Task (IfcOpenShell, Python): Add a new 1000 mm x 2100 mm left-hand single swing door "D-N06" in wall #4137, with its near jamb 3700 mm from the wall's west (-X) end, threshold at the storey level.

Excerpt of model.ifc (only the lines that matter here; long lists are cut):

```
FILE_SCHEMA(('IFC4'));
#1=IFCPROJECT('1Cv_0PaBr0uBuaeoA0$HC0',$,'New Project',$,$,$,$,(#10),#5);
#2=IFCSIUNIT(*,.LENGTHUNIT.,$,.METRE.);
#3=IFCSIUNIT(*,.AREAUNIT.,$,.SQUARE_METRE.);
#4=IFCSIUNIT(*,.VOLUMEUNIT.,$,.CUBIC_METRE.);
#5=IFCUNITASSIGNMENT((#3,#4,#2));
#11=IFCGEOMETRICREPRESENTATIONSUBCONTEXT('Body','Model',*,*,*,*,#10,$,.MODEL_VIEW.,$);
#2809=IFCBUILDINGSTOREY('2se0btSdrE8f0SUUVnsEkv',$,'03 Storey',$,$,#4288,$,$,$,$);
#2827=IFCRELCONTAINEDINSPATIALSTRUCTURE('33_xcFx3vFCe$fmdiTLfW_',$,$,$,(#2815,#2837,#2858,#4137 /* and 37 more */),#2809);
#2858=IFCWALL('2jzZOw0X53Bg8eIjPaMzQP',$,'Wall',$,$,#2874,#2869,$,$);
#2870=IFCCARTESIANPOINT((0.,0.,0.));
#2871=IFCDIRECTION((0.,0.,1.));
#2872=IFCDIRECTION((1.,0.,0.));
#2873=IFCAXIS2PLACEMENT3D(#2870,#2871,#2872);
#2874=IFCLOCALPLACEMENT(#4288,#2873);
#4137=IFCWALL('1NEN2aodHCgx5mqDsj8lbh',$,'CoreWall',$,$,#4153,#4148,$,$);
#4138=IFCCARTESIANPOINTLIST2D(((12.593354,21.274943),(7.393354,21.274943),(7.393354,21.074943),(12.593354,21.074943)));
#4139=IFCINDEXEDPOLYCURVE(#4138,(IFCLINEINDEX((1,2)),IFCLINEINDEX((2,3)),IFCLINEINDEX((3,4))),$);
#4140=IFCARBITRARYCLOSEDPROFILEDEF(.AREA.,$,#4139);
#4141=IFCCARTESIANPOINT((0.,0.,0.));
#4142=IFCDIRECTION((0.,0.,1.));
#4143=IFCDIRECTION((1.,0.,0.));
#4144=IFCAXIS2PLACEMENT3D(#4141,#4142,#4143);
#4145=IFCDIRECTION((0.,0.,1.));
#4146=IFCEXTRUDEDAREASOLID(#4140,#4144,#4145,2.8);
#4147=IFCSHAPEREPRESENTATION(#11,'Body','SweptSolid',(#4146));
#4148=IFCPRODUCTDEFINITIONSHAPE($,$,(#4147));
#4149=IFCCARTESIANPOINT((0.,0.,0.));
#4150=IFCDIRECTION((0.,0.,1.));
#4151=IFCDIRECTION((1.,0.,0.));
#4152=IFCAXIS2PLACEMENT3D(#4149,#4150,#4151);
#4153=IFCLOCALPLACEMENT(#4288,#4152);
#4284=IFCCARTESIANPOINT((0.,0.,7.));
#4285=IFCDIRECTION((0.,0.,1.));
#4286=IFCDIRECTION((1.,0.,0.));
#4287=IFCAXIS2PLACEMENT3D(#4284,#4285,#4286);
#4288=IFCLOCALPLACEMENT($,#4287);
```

```python
import numpy as np
import ifcopenshell
import ifcopenshell.api.feature
import ifcopenshell.api.geometry
import ifcopenshell.api.root
import ifcopenshell.api.spatial
import ifcopenshell.geom
import ifcopenshell.util.element
import ifcopenshell.util.placement
import ifcopenshell.util.representation
import ifcopenshell.util.shape
import ifcopenshell.util.unit

model = ifcopenshell.open("model.ifc")
unit_scale = ifcopenshell.util.unit.calculate_unit_scale(model)
settings = ifcopenshell.geom.settings()


def volume(element):
    """Net volume in cubic metres, openings subtracted."""
    shape = ifcopenshell.geom.create_shape(settings, element)
    return ifcopenshell.util.shape.get_volume(shape.geometry)


wall = model.by_id(4137)
storey = ifcopenshell.util.element.get_container(wall, ifc_class="IfcBuildingStorey")
context = ifcopenshell.util.representation.get_context(model, "Model", "Body", "MODEL_VIEW")
before = volume(wall)

width, height, from_end, sill = 1, 2.1, 3.7, 0.0  # metres

# The wall runs along its own X axis, and the end named is its -X end.
wall_shape = ifcopenshell.geom.create_shape(settings, wall)
x, y, z = ifcopenshell.util.shape.get_vertices(wall_shape.geometry).T
start = x.min() + from_end
face, thickness = float(y.min()), float(y.max() - y.min())
wall_matrix = ifcopenshell.util.placement.get_local_placement(wall.ObjectPlacement)
level = ifcopenshell.util.placement.get_local_placement(storey.ObjectPlacement)[2, 3]


def in_wall(x, y):
    """Placement at x, y metres in the wall's axes, at sill height."""
    matrix = wall_matrix.copy()
    matrix[:, 3] = wall_matrix @ np.array([x / unit_scale, y / unit_scale, 0.0, 1.0])
    matrix[2, 3] = level + sill / unit_scale
    return matrix


# Opening: a box that overshoots both wall faces by 50 mm.
opening = ifcopenshell.api.root.create_entity(model, ifc_class="IfcOpeningElement", predefined_type="OPENING")
box = ifcopenshell.api.geometry.add_wall_representation(
    model, context=context, length=width, height=height, thickness=thickness + 0.1
)
ifcopenshell.api.geometry.assign_representation(model, product=opening, representation=box)
ifcopenshell.api.geometry.edit_object_placement(model, product=opening, matrix=in_wall(start, face - 0.05), is_si=False)
ifcopenshell.api.feature.add_feature(model, feature=opening, element=wall)

door = ifcopenshell.api.root.create_entity(model, ifc_class="IfcDoor", name="D-N06", predefined_type="DOOR")
door.OverallWidth, door.OverallHeight = width / unit_scale, height / unit_scale
door.OperationType = "SINGLE_SWING_LEFT"
body = ifcopenshell.api.geometry.add_door_representation(
    model,
    context=context,
    overall_width=door.OverallWidth,
    overall_height=door.OverallHeight,
    operation_type="SINGLE_SWING_LEFT",
    lining_properties={"LiningDepth": thickness / unit_scale, "ThresholdDepth": thickness / unit_scale},
)
ifcopenshell.api.geometry.assign_representation(model, product=door, representation=body)
ifcopenshell.api.spatial.assign_container(model, products=[door], relating_structure=storey)
ifcopenshell.api.feature.add_filling(model, opening=opening, element=door)

# The lining spans the wall, so the door starts at the wall face.
ifcopenshell.api.geometry.edit_object_placement(model, product=door, matrix=in_wall(start, face), is_si=False)

after = volume(wall)

print(f"wall volume {before:.3f} -> {after:.3f} m3")

model.write("model_v2.ifc")
```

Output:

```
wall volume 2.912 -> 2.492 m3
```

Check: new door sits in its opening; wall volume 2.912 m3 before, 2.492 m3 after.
